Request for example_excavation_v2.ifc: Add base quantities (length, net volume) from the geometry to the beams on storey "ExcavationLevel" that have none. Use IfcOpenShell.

First a look at what the model holds.

```python
import ifcopenshell
import ifcopenshell.util.element
import ifcopenshell.util.unit

model = ifcopenshell.open("example_excavation_v2.ifc")
print(model.schema)
for unit_type in ("LENGTHUNIT", "AREAUNIT", "VOLUMEUNIT"):
    print(unit_type, ifcopenshell.util.unit.calculate_unit_scale(model, unit_type))
storey = next(s for s in model.by_type("IfcBuildingStorey") if s.Name == "ExcavationLevel")
beams = [e for e in ifcopenshell.util.element.get_decomposition(storey) if e.is_a("IfcBeam")]
for e in sorted(beams, key=lambda e: e.id()):
    print(e.id(), e.is_a(), e.Name, list(ifcopenshell.util.element.get_psets(e, qtos_only=True)), sep=" | ")
```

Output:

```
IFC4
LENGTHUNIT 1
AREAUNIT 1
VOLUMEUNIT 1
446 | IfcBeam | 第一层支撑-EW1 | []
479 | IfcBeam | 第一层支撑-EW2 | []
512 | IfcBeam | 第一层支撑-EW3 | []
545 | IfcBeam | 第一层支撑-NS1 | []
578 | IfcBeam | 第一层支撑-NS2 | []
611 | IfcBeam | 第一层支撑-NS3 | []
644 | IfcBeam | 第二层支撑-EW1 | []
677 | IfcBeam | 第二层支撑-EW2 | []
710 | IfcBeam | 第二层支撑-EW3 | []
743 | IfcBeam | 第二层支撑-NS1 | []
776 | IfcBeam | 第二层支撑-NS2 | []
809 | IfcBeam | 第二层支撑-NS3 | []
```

```python
import ifcopenshell
import ifcopenshell.api.pset
import ifcopenshell.geom
import ifcopenshell.util.element
import ifcopenshell.util.shape
import ifcopenshell.util.unit

model = ifcopenshell.open("example_excavation_v2.ifc")
unit_scale = ifcopenshell.util.unit.calculate_unit_scale(model)
volume_scale = ifcopenshell.util.unit.calculate_unit_scale(model, "VOLUMEUNIT")
settings = ifcopenshell.geom.settings()

storey = next(s for s in model.by_type("IfcBuildingStorey") if s.Name == "ExcavationLevel")
beams = [e for e in ifcopenshell.util.element.get_decomposition(storey) if e.is_a("IfcBeam")]

for e in sorted(beams, key=lambda e: e.id()):
    if ifcopenshell.util.element.get_psets(e, qtos_only=True, should_inherit=False):
        continue
    # Geometry comes back in metres, in the element's own axes.
    shape = ifcopenshell.geom.create_shape(settings, e)
    values = {
        "Length": ifcopenshell.util.shape.get_max_xyz(shape.geometry) / unit_scale,
        "NetVolume": ifcopenshell.util.shape.get_volume(shape.geometry) / volume_scale,
    }
    qto = ifcopenshell.api.pset.add_qto(model, product=e, name="Qto_BeamBaseQuantities")
    ifcopenshell.api.pset.edit_qto(model, qto=qto, properties=values)
    print(e.id(), {k: round(v, 3) for k, v in values.items()})

model.write("example_excavation_v2_rev.ifc")
```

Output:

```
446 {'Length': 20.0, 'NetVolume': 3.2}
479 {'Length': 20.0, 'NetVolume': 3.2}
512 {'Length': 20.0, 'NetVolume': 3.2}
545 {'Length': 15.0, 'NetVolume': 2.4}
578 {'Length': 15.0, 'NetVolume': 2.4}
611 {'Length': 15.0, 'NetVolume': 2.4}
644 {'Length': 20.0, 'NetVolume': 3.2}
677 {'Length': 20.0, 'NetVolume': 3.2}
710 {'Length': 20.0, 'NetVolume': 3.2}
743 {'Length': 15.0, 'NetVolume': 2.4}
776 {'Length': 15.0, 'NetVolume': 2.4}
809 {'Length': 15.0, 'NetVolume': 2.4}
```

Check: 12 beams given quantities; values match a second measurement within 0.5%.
